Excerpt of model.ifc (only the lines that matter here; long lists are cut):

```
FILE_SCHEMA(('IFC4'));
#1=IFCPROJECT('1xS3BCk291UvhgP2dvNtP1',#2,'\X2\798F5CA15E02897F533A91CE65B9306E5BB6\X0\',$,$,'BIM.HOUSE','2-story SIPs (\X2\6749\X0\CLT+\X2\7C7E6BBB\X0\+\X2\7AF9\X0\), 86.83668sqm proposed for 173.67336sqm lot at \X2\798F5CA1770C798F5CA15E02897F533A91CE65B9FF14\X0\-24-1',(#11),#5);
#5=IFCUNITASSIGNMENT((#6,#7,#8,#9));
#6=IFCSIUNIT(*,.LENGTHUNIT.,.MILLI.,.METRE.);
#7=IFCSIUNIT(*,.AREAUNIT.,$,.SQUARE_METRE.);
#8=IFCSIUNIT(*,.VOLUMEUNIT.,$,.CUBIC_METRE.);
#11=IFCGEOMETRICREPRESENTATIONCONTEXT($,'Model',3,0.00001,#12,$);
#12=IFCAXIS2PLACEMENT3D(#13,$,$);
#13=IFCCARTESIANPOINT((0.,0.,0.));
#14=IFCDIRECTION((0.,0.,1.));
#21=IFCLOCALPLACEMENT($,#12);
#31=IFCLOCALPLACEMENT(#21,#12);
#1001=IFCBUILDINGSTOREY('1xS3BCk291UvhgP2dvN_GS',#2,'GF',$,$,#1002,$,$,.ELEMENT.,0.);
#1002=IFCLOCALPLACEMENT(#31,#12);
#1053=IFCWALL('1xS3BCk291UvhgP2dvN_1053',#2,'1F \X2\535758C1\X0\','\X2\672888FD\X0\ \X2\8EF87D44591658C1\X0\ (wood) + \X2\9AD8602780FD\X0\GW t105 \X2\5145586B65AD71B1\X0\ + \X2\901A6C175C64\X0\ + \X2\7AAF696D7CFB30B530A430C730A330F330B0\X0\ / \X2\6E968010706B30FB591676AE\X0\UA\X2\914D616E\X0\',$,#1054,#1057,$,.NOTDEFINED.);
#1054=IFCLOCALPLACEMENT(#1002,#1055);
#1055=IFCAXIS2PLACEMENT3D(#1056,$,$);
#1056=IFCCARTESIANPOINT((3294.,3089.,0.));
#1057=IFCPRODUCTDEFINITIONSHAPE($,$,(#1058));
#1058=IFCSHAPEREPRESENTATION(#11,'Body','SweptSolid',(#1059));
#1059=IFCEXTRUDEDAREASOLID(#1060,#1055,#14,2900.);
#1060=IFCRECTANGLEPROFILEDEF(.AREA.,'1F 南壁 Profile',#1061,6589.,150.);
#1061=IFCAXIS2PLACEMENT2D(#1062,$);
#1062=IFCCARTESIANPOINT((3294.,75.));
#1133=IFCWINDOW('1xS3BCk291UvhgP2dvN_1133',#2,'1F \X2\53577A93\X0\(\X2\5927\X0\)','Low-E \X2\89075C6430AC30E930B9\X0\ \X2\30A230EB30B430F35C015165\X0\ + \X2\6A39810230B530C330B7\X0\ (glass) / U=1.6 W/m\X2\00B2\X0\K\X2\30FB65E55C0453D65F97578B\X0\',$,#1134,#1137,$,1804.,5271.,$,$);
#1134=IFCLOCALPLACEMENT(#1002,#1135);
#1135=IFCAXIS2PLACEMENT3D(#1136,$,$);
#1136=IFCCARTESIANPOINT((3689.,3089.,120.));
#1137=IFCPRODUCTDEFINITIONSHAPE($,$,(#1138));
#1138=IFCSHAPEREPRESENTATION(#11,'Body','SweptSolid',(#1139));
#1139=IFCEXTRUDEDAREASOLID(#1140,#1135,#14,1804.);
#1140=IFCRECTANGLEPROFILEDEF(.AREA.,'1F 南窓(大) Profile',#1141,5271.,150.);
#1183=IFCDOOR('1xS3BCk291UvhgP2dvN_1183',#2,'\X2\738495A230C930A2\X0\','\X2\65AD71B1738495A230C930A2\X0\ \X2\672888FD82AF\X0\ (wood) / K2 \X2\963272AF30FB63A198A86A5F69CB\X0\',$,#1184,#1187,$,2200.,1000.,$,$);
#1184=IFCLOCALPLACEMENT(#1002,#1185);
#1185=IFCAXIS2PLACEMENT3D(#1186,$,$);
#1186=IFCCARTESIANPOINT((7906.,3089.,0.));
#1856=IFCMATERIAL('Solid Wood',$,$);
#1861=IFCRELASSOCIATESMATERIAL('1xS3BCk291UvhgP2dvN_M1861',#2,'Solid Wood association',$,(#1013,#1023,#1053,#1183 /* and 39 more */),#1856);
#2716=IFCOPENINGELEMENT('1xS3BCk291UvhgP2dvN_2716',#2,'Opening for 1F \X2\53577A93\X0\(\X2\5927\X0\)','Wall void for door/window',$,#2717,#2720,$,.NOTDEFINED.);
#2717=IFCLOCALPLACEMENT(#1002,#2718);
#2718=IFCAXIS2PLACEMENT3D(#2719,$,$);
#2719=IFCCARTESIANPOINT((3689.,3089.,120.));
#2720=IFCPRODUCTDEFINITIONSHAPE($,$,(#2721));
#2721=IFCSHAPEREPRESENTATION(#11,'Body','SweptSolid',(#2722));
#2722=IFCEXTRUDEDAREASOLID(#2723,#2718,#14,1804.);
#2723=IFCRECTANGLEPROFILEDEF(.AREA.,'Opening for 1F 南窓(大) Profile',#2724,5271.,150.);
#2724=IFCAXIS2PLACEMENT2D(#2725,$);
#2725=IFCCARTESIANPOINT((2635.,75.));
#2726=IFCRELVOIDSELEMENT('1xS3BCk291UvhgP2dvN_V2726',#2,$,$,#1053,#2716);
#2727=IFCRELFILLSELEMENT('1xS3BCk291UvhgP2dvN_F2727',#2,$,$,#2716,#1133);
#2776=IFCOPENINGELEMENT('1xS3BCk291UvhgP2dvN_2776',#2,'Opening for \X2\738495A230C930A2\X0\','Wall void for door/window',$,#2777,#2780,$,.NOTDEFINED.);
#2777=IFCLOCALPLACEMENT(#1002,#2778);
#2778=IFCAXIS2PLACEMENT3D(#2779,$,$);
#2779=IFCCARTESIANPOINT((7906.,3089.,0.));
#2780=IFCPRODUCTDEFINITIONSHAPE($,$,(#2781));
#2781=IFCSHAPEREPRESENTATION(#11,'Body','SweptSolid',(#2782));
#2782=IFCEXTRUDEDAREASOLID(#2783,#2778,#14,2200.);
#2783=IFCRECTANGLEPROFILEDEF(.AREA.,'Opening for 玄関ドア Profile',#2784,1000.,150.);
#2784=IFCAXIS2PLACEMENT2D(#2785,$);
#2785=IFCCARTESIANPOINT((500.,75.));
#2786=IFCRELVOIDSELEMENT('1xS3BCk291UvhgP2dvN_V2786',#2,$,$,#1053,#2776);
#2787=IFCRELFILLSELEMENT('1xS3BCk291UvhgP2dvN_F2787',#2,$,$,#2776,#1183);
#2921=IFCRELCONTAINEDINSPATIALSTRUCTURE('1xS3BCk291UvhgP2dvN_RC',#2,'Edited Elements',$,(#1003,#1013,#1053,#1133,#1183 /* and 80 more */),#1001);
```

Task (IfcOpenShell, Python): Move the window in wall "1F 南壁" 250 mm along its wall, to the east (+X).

```python
import ifcopenshell
import ifcopenshell.api.geometry
import ifcopenshell.util.placement
import ifcopenshell.util.unit

model = ifcopenshell.open("model.ifc")
unit_scale = ifcopenshell.util.unit.calculate_unit_scale(model)

window = model.by_guid("1xS3BCk291UvhgP2dvN_1133")
opening = window.FillsVoids[0].RelatingOpeningElement
wall = opening.VoidsElements[0].RelatingBuildingElement

wall_matrix = ifcopenshell.util.placement.get_local_placement(wall.ObjectPlacement)
shift = wall_matrix[:3, 0] * 0.25 / unit_scale
before = ifcopenshell.util.placement.get_local_placement(window.ObjectPlacement)[:3, 3].copy()

# The window is not placed relative to its opening, so move both.
for product in (opening, window):
    matrix = ifcopenshell.util.placement.get_local_placement(product.ObjectPlacement)
    matrix[:3, 3] += shift
    ifcopenshell.api.geometry.edit_object_placement(model, product=product, matrix=matrix, is_si=False)

after = ifcopenshell.util.placement.get_local_placement(window.ObjectPlacement)[:3, 3]
print("window moved by", (after - before).round(3) + 0.0)

model.write("model_v2.ifc")
```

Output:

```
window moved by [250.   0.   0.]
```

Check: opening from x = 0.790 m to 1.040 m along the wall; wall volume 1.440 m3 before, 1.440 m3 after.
